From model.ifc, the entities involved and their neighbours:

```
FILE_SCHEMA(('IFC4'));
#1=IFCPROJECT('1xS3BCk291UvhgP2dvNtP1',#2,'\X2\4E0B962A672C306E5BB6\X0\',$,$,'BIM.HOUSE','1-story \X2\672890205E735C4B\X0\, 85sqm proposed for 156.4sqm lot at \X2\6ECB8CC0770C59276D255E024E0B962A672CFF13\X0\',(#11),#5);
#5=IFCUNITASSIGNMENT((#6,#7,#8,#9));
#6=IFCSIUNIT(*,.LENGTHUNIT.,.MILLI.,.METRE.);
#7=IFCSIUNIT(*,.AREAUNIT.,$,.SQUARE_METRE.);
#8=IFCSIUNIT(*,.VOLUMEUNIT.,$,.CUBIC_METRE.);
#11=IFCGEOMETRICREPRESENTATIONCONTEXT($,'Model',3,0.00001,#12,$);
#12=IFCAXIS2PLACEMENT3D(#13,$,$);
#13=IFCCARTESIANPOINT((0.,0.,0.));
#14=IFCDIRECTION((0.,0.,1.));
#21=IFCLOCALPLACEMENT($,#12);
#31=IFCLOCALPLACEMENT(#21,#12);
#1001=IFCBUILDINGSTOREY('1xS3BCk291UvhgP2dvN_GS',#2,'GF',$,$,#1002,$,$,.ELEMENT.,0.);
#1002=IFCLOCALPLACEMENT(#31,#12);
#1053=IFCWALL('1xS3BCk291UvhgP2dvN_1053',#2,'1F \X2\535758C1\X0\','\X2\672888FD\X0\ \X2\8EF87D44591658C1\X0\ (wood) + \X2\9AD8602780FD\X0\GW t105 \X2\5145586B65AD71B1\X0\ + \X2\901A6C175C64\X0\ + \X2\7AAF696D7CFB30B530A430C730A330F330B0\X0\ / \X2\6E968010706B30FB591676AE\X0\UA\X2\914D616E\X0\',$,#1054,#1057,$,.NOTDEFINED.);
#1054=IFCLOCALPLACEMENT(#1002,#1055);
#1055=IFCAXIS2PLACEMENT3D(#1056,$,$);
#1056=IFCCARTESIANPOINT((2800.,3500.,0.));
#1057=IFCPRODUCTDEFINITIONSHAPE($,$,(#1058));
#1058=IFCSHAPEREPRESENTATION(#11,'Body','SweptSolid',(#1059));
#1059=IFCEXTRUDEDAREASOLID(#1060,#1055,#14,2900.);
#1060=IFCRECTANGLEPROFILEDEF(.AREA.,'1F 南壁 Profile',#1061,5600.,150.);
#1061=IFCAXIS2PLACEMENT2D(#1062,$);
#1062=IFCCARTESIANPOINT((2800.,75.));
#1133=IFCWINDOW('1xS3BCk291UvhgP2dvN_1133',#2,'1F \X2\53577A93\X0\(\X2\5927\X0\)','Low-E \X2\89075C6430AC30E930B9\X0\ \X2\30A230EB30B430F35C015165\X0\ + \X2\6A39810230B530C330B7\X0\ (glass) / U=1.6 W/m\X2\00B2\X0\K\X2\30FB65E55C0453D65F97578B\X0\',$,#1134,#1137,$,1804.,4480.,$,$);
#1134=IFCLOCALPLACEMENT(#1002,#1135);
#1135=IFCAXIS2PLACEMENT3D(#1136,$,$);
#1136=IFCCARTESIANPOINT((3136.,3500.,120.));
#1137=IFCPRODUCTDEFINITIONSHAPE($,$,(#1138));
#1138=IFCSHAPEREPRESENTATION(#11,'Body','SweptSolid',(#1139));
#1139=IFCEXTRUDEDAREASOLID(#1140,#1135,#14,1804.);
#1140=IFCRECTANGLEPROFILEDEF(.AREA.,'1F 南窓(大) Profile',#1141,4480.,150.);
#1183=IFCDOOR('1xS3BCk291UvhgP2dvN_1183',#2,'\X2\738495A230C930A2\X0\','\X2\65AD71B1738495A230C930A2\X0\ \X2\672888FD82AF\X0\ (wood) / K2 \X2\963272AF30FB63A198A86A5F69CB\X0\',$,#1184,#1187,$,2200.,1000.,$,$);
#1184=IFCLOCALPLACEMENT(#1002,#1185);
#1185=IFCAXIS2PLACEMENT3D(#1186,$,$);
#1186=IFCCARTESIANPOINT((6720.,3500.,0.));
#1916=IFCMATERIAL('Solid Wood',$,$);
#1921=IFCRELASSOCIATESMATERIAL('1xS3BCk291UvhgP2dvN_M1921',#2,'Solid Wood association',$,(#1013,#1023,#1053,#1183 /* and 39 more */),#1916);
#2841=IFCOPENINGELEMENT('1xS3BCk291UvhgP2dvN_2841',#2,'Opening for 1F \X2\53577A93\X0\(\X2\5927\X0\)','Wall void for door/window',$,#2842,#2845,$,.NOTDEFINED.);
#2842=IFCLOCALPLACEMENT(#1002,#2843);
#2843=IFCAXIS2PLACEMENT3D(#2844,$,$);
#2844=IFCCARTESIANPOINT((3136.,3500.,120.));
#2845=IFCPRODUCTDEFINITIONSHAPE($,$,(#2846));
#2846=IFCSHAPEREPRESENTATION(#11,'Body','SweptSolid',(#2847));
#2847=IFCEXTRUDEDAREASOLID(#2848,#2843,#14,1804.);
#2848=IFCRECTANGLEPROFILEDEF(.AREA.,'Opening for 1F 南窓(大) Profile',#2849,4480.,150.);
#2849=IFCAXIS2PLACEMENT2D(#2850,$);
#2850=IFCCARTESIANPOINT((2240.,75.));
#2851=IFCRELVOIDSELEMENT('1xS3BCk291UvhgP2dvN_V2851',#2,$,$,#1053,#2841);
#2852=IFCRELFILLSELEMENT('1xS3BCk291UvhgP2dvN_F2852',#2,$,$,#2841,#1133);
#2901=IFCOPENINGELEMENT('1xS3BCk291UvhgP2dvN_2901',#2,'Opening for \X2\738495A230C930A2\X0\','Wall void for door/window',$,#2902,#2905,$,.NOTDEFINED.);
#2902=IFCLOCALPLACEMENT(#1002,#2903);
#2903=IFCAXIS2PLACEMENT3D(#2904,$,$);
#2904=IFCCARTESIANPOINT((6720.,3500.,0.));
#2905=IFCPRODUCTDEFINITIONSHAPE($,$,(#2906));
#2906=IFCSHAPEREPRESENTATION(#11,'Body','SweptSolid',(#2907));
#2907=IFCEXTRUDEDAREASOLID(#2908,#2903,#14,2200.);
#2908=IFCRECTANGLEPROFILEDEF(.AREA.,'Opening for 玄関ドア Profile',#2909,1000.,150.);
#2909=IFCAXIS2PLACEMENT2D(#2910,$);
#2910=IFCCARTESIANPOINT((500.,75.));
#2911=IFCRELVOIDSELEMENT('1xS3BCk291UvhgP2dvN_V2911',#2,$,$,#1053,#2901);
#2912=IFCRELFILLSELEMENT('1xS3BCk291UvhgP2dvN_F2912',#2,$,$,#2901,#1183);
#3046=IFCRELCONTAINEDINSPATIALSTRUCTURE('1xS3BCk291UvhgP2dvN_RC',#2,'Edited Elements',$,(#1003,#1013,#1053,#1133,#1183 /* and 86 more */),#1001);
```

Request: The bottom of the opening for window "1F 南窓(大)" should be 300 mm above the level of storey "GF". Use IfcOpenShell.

```python
import numpy as np
import ifcopenshell
import ifcopenshell.api.geometry
import ifcopenshell.geom
import ifcopenshell.util.element
import ifcopenshell.util.placement
import ifcopenshell.util.shape
import ifcopenshell.util.unit

model = ifcopenshell.open("model.ifc")
unit_scale = ifcopenshell.util.unit.calculate_unit_scale(model)

window = model.by_id(1133)
opening = window.FillsVoids[0].RelatingOpeningElement
storey = ifcopenshell.util.element.get_container(window, ifc_class="IfcBuildingStorey")
level = ifcopenshell.util.placement.get_local_placement(storey.ObjectPlacement)[2, 3]

# The opening's origin need not be at the sill, so measure its lowest point.
shape = ifcopenshell.geom.create_shape(ifcopenshell.geom.settings(), opening)
bottom = ifcopenshell.util.shape.get_shape_bottom_elevation(shape, shape.geometry) / unit_scale
dz = level + 0.3 / unit_scale - bottom

shift = np.array([0.0, 0.0, dz])
# The window is not placed relative to its opening, so move both.
for product in (opening, window):
    matrix = ifcopenshell.util.placement.get_local_placement(product.ObjectPlacement)
    matrix[:3, 3] += shift
    ifcopenshell.api.geometry.edit_object_placement(model, product=product, matrix=matrix, is_si=False)

print(f"moved by {dz * unit_scale:+.3f} m")

model.write("model_updated.ifc")
```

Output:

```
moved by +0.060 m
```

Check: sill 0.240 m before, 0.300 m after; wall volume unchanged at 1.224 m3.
